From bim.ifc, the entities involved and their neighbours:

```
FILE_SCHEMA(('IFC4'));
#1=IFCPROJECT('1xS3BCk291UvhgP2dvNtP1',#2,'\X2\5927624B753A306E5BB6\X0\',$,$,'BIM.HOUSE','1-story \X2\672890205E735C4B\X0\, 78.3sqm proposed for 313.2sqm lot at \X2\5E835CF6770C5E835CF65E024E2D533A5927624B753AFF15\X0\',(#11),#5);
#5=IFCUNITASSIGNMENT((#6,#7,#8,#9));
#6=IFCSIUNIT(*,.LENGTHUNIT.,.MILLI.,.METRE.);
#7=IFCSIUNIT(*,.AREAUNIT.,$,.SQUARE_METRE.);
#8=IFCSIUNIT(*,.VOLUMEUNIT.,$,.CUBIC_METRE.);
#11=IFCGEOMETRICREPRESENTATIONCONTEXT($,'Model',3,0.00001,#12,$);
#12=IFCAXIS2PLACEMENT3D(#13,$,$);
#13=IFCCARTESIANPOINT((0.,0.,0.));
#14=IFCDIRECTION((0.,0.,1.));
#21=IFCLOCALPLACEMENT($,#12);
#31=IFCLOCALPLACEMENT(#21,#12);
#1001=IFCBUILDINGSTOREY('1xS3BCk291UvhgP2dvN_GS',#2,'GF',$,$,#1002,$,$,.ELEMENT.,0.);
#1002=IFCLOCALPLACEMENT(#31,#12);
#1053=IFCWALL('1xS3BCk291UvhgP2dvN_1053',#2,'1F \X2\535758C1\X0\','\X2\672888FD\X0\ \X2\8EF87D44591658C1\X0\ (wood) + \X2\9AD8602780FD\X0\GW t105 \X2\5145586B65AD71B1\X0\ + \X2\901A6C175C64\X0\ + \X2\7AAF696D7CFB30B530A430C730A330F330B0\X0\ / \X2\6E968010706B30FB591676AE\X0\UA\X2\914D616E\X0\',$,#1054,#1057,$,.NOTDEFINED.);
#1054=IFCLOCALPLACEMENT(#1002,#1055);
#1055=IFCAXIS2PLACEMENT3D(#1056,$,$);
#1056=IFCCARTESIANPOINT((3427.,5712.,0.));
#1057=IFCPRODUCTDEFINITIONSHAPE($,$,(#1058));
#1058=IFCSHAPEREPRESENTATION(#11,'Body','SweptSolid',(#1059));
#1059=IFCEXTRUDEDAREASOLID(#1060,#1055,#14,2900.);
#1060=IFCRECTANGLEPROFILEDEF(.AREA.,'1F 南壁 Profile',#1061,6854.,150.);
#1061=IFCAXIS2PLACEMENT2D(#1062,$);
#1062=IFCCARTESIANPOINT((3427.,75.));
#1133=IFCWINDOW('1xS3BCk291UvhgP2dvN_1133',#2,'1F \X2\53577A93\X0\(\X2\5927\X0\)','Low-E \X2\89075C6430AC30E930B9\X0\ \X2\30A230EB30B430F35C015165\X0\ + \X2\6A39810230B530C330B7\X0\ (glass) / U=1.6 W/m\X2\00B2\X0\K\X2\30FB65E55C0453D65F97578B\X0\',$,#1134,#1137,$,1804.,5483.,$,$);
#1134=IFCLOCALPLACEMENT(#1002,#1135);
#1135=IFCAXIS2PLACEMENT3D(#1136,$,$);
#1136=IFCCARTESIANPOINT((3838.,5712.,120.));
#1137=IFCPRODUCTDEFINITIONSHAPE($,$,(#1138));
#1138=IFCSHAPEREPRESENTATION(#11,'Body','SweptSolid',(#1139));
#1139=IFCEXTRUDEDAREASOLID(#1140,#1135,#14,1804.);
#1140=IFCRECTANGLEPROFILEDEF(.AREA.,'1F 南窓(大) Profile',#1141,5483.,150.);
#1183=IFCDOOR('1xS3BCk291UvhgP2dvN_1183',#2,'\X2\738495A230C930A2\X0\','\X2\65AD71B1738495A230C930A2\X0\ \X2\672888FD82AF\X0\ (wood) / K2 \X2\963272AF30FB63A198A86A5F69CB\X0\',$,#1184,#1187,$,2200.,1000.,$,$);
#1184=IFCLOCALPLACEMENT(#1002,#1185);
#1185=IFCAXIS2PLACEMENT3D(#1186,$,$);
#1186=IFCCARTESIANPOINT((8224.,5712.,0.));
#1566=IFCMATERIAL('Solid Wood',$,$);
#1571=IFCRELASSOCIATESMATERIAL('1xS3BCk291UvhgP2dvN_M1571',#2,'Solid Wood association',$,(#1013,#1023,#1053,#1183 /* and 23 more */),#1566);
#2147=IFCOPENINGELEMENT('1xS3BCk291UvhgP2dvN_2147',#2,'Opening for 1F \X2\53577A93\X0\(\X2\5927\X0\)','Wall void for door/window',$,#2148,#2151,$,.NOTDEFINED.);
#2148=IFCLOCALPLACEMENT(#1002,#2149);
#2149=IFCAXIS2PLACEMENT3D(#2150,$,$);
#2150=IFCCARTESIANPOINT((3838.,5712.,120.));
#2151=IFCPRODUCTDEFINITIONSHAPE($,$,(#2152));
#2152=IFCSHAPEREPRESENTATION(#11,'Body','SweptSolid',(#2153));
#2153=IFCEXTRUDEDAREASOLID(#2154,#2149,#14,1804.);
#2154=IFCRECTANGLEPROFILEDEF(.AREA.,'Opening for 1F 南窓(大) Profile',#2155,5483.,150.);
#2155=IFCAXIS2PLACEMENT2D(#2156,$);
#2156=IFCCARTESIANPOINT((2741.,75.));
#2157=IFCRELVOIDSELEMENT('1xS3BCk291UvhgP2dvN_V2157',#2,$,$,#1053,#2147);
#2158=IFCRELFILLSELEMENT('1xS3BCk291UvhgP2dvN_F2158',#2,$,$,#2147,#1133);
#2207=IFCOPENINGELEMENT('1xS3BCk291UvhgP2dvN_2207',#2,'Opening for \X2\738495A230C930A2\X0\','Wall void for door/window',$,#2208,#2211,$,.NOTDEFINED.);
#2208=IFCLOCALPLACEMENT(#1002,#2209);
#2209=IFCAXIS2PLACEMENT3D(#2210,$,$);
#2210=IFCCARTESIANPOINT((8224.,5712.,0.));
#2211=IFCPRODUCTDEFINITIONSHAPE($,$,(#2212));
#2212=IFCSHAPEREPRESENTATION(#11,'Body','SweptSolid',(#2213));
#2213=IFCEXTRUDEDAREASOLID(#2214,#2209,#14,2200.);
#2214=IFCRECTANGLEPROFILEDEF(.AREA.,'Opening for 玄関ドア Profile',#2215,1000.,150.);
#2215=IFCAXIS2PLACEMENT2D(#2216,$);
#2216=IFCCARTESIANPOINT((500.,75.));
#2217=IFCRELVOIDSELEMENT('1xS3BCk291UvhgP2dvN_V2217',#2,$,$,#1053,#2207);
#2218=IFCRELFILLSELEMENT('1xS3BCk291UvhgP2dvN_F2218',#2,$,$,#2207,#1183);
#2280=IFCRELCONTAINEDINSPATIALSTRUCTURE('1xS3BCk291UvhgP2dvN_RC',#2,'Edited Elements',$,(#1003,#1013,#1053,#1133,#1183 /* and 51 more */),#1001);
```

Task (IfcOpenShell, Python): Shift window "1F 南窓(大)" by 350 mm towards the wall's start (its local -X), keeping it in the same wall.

```python
import ifcopenshell
import ifcopenshell.api.geometry
import ifcopenshell.util.placement
import ifcopenshell.util.unit

model = ifcopenshell.open("bim.ifc")
unit_scale = ifcopenshell.util.unit.calculate_unit_scale(model)

window = model.by_guid("1xS3BCk291UvhgP2dvN_1133")
opening = window.FillsVoids[0].RelatingOpeningElement
wall = opening.VoidsElements[0].RelatingBuildingElement

wall_matrix = ifcopenshell.util.placement.get_local_placement(wall.ObjectPlacement)
shift = wall_matrix[:3, 0] * -0.35 / unit_scale
before = ifcopenshell.util.placement.get_local_placement(window.ObjectPlacement)[:3, 3].copy()

# The window is not placed relative to its opening, so move both.
for product in (opening, window):
    matrix = ifcopenshell.util.placement.get_local_placement(product.ObjectPlacement)
    matrix[:3, 3] += shift
    ifcopenshell.api.geometry.edit_object_placement(model, product=product, matrix=matrix, is_si=False)

after = ifcopenshell.util.placement.get_local_placement(window.ObjectPlacement)[:3, 3]
print("window moved by", (after - before).round(3) + 0.0)

model.write("bim_updated.ifc")
```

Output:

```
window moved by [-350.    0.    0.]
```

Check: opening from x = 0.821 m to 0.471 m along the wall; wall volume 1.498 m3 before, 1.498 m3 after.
